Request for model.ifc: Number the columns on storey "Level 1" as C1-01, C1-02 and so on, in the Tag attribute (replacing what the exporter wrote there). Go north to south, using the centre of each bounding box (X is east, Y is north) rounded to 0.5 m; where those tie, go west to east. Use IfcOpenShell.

First a look at what the model holds.

```python
import ifcopenshell
import ifcopenshell.util.element
import ifcopenshell.util.placement

model = ifcopenshell.open("model.ifc")
print(model.schema)
storey = next(s for s in model.by_type("IfcBuildingStorey") if s.Name == "Level 1")
columns = [e for e in ifcopenshell.util.element.get_decomposition(storey) if e.is_a("IfcColumn")]
for e in sorted(columns, key=lambda e: e.id()):
    origin = ifcopenshell.util.placement.get_local_placement(e.ObjectPlacement)[:3, 3]
    print(e.id(), e.Tag, e.Name, origin.round(2) + 0.0, sep=" | ")
```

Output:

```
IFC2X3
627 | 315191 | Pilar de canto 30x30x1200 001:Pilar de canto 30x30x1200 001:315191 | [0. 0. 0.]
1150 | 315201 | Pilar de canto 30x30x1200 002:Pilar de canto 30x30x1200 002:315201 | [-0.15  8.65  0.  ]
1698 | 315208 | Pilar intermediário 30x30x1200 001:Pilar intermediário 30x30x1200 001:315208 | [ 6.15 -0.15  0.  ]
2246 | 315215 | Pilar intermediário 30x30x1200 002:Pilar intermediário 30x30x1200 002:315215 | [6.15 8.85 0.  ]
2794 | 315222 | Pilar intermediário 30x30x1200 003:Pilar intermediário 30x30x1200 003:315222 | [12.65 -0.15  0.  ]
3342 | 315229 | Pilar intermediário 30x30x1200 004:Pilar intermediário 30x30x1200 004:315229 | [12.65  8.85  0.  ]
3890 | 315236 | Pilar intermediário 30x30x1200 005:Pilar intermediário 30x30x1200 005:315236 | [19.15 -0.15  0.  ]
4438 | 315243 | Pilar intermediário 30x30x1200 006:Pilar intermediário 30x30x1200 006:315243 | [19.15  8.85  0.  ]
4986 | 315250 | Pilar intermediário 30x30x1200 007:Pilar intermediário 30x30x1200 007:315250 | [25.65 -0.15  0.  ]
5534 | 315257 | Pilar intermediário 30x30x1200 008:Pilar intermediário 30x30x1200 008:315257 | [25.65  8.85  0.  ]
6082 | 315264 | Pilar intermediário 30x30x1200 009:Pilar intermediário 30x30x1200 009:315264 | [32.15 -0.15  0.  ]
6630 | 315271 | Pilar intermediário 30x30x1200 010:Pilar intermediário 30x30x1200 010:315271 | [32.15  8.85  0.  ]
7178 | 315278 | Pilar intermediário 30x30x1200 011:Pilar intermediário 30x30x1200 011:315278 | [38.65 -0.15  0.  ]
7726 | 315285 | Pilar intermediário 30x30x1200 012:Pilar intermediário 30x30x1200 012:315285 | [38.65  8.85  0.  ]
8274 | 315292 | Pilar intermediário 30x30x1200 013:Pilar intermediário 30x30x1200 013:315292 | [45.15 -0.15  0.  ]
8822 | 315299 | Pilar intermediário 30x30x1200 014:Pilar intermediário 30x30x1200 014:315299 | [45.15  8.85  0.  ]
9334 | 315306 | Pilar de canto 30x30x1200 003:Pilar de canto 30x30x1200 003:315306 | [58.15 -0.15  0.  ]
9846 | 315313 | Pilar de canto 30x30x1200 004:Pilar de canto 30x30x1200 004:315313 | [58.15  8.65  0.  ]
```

```python
import ifcopenshell
import ifcopenshell.geom
import ifcopenshell.util.element
import ifcopenshell.util.shape

model = ifcopenshell.open("model.ifc")
settings = ifcopenshell.geom.settings()
settings.set("use-world-coords", True)


def centre(element):
    shape = ifcopenshell.geom.create_shape(settings, element)
    return ifcopenshell.util.shape.get_bbox_centroid(shape.geometry)


storey = next(s for s in model.by_type("IfcBuildingStorey") if s.Name == "Level 1")
columns = [e for e in ifcopenshell.util.element.get_decomposition(storey) if e.is_a("IfcColumn")]

# Insertion points can sit at a corner or the storey origin, so sort by the geometry (in metres).
centres = {e: centre(e) for e in columns}
columns.sort(key=lambda e: (-round(centres[e][1] / 0.5), centres[e][0]))

for i, e in enumerate(columns, start=1):
    number = f"C1-{i:02d}"
    e.Tag = number
    print(e.id(), number)

model.write("model-out.ifc")
```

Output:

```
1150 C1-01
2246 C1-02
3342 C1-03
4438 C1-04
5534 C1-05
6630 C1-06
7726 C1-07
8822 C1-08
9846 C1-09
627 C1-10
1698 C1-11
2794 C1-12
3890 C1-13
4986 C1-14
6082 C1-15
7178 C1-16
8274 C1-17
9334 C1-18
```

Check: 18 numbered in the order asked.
